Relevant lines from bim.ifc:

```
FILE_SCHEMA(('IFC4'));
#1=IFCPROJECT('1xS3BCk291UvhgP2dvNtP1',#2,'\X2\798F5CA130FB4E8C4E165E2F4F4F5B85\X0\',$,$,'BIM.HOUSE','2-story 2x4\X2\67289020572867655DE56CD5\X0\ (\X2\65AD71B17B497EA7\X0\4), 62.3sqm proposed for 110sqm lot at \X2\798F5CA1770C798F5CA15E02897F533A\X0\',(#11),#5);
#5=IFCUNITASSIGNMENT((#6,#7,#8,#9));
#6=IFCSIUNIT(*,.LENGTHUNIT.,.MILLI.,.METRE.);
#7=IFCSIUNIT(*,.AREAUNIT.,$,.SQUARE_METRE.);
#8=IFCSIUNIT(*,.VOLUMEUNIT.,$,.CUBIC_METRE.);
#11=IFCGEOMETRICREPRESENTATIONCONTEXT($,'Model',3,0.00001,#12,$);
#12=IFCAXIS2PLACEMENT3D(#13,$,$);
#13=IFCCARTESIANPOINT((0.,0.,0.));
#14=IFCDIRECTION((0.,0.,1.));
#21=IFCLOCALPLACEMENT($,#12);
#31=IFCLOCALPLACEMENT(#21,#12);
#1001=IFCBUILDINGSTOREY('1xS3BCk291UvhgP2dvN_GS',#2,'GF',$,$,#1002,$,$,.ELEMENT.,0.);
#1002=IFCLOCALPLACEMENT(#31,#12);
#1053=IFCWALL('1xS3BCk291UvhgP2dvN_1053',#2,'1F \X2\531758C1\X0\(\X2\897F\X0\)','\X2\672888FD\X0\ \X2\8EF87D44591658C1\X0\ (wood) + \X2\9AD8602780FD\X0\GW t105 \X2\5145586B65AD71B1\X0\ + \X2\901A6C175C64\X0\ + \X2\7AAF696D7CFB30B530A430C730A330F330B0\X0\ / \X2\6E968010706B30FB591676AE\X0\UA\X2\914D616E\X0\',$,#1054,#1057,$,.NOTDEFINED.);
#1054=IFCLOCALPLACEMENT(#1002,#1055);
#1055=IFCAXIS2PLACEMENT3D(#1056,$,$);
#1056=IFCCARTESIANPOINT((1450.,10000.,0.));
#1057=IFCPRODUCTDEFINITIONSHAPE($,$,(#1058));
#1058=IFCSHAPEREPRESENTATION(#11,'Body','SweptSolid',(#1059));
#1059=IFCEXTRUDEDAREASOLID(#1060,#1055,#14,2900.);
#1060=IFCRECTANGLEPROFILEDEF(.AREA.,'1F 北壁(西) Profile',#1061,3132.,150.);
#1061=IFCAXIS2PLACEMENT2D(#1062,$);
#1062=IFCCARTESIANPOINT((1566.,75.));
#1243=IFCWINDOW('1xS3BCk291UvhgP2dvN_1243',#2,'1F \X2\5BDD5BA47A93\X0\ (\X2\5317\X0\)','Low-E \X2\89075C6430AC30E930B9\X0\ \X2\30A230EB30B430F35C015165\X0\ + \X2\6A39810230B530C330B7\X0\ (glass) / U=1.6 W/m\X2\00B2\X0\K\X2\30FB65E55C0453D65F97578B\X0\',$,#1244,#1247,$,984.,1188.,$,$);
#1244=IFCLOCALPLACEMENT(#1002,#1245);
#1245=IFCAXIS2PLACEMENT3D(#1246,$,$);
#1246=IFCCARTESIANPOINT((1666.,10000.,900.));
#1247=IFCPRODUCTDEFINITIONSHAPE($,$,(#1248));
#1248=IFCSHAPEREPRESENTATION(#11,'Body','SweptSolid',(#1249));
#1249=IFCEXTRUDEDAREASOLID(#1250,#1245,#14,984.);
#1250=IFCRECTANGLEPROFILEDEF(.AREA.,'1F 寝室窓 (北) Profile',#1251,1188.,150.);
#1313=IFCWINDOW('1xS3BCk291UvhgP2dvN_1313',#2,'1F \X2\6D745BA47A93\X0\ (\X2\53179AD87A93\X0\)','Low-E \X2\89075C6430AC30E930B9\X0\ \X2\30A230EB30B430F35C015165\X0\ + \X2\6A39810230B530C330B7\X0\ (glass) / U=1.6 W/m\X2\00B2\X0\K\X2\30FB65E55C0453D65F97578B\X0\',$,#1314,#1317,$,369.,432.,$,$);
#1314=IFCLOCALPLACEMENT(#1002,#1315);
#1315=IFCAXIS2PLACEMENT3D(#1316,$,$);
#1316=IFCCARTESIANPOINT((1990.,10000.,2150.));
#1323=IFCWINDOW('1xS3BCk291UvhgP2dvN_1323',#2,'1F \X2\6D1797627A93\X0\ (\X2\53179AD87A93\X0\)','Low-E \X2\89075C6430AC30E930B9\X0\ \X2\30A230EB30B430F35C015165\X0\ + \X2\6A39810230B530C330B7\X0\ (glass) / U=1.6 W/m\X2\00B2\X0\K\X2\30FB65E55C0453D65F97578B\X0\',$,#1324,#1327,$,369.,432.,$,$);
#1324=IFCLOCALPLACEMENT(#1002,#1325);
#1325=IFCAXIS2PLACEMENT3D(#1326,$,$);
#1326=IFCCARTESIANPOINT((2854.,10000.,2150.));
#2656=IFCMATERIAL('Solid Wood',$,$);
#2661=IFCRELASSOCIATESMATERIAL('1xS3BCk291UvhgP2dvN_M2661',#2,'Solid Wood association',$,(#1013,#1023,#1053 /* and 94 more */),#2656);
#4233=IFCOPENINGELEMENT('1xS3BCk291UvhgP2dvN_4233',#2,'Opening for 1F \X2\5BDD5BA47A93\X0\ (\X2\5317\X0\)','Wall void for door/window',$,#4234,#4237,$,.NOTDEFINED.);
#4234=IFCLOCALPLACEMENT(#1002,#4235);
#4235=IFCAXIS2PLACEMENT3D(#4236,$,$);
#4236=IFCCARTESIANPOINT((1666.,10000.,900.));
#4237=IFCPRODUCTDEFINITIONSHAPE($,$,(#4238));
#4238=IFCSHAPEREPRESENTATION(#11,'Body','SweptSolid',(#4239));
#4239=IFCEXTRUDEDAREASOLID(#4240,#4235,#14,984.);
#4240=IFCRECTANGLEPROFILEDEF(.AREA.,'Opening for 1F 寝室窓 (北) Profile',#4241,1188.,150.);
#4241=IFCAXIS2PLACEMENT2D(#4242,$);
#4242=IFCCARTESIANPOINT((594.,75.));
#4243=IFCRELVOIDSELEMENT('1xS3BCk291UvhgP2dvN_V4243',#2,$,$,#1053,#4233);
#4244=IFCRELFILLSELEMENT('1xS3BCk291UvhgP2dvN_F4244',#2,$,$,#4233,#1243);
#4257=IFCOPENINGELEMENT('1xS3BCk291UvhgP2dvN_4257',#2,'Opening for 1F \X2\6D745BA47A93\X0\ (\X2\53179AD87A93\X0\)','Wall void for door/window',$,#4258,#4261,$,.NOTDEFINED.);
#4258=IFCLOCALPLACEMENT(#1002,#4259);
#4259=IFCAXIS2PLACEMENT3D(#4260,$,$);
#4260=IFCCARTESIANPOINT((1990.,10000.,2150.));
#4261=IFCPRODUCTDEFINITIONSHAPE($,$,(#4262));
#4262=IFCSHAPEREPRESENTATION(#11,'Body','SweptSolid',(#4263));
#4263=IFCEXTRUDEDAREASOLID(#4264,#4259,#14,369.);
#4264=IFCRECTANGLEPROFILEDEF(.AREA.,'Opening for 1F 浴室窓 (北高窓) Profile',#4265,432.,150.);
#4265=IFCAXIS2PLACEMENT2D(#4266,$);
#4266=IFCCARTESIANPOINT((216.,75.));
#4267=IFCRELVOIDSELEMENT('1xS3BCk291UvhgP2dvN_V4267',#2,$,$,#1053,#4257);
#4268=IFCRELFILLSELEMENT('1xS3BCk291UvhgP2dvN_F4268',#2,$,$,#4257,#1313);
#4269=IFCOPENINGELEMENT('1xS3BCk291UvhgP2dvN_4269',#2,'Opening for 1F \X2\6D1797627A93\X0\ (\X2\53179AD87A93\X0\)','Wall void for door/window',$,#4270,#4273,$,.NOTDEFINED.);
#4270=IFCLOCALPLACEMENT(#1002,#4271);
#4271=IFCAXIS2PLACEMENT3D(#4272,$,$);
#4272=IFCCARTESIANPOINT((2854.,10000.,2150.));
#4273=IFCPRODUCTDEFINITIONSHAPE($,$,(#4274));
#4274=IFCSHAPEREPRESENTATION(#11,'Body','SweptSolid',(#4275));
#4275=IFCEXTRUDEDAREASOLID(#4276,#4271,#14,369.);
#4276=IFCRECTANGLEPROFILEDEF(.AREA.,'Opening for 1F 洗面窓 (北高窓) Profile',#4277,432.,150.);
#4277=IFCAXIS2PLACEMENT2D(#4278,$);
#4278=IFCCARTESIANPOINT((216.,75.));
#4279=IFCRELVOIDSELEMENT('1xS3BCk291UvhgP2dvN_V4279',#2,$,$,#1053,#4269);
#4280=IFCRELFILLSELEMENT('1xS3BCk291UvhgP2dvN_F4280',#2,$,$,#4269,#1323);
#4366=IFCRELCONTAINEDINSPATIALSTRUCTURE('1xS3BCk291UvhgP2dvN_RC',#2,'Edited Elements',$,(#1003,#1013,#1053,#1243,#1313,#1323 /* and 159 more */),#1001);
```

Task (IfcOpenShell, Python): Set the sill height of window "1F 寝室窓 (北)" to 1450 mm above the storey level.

```python
import numpy as np
import ifcopenshell
import ifcopenshell.api.geometry
import ifcopenshell.geom
import ifcopenshell.util.element
import ifcopenshell.util.placement
import ifcopenshell.util.shape
import ifcopenshell.util.unit

model = ifcopenshell.open("bim.ifc")
unit_scale = ifcopenshell.util.unit.calculate_unit_scale(model)

window = model.by_guid("1xS3BCk291UvhgP2dvN_1243")
opening = window.FillsVoids[0].RelatingOpeningElement
storey = ifcopenshell.util.element.get_container(window, ifc_class="IfcBuildingStorey")
level = ifcopenshell.util.placement.get_local_placement(storey.ObjectPlacement)[2, 3]

# The opening's origin need not be at the sill, so measure its lowest point.
shape = ifcopenshell.geom.create_shape(ifcopenshell.geom.settings(), opening)
bottom = ifcopenshell.util.shape.get_shape_bottom_elevation(shape, shape.geometry) / unit_scale
dz = level + 1450.0 - bottom

shift = np.array([0.0, 0.0, dz])
# The window is not placed relative to its opening, so move both.
for product in (opening, window):
    matrix = ifcopenshell.util.placement.get_local_placement(product.ObjectPlacement)
    matrix[:3, 3] += shift
    ifcopenshell.api.geometry.edit_object_placement(model, product=product, matrix=matrix, is_si=False)

print(f"moved by {dz * unit_scale:+.3f} m")

model.write("bim_updated.ifc")
```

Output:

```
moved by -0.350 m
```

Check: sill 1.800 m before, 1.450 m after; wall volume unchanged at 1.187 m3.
